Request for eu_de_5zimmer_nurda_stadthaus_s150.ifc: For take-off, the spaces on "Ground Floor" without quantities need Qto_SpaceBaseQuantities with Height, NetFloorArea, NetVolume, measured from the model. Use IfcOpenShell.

First a look at what the model holds.

```python
import ifcopenshell
import ifcopenshell.util.element
import ifcopenshell.util.unit

model = ifcopenshell.open("eu_de_5zimmer_nurda_stadthaus_s150.ifc")
print(model.schema)
for unit_type in ("LENGTHUNIT", "AREAUNIT", "VOLUMEUNIT"):
    print(unit_type, ifcopenshell.util.unit.calculate_unit_scale(model, unit_type))
storey = next(s for s in model.by_type("IfcBuildingStorey") if s.Name == "Ground Floor")
spaces = [e for e in ifcopenshell.util.element.get_decomposition(storey) if e.is_a("IfcSpace")]
for e in sorted(spaces, key=lambda e: e.id()):
    print(e.id(), e.is_a(), e.Name, list(ifcopenshell.util.element.get_psets(e, qtos_only=True)), sep=" | ")
```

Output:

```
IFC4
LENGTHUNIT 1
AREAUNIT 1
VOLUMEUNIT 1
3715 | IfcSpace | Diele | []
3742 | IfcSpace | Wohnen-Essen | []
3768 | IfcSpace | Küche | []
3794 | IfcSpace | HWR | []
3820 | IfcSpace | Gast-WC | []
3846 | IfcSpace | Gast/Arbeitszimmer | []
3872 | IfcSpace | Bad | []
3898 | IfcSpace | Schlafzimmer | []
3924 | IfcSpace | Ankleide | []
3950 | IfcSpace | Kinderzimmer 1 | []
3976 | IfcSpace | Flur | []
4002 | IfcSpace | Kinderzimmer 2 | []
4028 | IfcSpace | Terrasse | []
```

```python
import ifcopenshell
import ifcopenshell.api.pset
import ifcopenshell.geom
import ifcopenshell.util.element
import ifcopenshell.util.shape
import ifcopenshell.util.unit

model = ifcopenshell.open("eu_de_5zimmer_nurda_stadthaus_s150.ifc")
unit_scale = ifcopenshell.util.unit.calculate_unit_scale(model)
area_scale = ifcopenshell.util.unit.calculate_unit_scale(model, "AREAUNIT")
volume_scale = ifcopenshell.util.unit.calculate_unit_scale(model, "VOLUMEUNIT")
settings = ifcopenshell.geom.settings()

storey = next(s for s in model.by_type("IfcBuildingStorey") if s.Name == "Ground Floor")
spaces = [e for e in ifcopenshell.util.element.get_decomposition(storey) if e.is_a("IfcSpace")]

for e in sorted(spaces, key=lambda e: e.id()):
    if ifcopenshell.util.element.get_psets(e, qtos_only=True, should_inherit=False):
        continue
    # Geometry comes back in metres, in the element's own axes.
    shape = ifcopenshell.geom.create_shape(settings, e)
    values = {
        "Height": ifcopenshell.util.shape.get_z(shape.geometry) / unit_scale,
        "NetFloorArea": ifcopenshell.util.shape.get_footprint_area(shape.geometry) / area_scale,
        "NetVolume": ifcopenshell.util.shape.get_volume(shape.geometry) / volume_scale,
    }
    qto = ifcopenshell.api.pset.add_qto(model, product=e, name="Qto_SpaceBaseQuantities")
    ifcopenshell.api.pset.edit_qto(model, qto=qto, properties=values)
    print(e.id(), {k: round(v, 3) for k, v in values.items()})

model.write("eu_de_5zimmer_nurda_stadthaus_s150-out.ifc")
```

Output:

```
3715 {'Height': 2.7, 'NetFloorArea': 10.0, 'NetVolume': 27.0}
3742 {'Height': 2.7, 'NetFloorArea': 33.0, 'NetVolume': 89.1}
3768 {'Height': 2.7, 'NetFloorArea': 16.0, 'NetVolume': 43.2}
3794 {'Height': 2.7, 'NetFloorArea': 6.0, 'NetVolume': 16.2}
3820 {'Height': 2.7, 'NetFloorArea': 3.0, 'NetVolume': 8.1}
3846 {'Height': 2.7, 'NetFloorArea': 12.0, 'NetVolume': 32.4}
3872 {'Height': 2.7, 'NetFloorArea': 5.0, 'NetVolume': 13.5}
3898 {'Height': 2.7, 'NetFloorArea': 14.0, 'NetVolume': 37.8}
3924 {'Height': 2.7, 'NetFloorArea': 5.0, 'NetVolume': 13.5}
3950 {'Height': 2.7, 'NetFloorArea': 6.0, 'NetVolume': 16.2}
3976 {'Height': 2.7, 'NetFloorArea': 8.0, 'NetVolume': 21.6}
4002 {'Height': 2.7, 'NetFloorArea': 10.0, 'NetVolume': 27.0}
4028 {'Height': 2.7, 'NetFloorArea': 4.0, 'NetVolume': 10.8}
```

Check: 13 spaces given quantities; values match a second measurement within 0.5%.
